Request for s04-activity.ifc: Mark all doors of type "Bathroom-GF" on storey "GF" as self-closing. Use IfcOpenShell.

First a look at what the model holds.

```python
import ifcopenshell
import ifcopenshell.util.element

model = ifcopenshell.open("s04-activity.ifc")
print(model.schema)
storey = next(s for s in model.by_type("IfcBuildingStorey") if s.Name == "GF")
doors = [e for e in ifcopenshell.util.element.get_decomposition(storey) if e.is_a("IfcDoor")]
seen = {}
for e in doors:
    element_type = ifcopenshell.util.element.get_type(e)
    key = (element_type.Name if element_type != e and element_type else None, ifcopenshell.util.element.get_pset(e, "Pset_DoorCommon", "SelfClosing"))
    seen[key] = seen.get(key, 0) + 1
for (name, value), count in sorted(seen.items(), key=str):
    print(count, "x", name, "|", value)
```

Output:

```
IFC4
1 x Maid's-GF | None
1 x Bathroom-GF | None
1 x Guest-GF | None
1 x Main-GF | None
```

```python
import ifcopenshell
import ifcopenshell.api.pset
import ifcopenshell.util.element

model = ifcopenshell.open("s04-activity.ifc")

storey = next(s for s in model.by_type("IfcBuildingStorey") if s.Name == "GF")
doors = [e for e in ifcopenshell.util.element.get_decomposition(storey) if e.is_a("IfcDoor")]

count = 0
for e in doors:
    element_type = ifcopenshell.util.element.get_type(e)
    if element_type in (None, e) or element_type.Name != "Bathroom-GF":
        continue
    # add_pset returns the element's existing set when there is one.
    pset = ifcopenshell.api.pset.add_pset(model, product=e, name="Pset_DoorCommon")
    ifcopenshell.api.pset.edit_pset(model, pset=pset, properties={"SelfClosing": True})
    count += 1

print(count, "doors updated")

model.write("s04-activity_updated.ifc")
```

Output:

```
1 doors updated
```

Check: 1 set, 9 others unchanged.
